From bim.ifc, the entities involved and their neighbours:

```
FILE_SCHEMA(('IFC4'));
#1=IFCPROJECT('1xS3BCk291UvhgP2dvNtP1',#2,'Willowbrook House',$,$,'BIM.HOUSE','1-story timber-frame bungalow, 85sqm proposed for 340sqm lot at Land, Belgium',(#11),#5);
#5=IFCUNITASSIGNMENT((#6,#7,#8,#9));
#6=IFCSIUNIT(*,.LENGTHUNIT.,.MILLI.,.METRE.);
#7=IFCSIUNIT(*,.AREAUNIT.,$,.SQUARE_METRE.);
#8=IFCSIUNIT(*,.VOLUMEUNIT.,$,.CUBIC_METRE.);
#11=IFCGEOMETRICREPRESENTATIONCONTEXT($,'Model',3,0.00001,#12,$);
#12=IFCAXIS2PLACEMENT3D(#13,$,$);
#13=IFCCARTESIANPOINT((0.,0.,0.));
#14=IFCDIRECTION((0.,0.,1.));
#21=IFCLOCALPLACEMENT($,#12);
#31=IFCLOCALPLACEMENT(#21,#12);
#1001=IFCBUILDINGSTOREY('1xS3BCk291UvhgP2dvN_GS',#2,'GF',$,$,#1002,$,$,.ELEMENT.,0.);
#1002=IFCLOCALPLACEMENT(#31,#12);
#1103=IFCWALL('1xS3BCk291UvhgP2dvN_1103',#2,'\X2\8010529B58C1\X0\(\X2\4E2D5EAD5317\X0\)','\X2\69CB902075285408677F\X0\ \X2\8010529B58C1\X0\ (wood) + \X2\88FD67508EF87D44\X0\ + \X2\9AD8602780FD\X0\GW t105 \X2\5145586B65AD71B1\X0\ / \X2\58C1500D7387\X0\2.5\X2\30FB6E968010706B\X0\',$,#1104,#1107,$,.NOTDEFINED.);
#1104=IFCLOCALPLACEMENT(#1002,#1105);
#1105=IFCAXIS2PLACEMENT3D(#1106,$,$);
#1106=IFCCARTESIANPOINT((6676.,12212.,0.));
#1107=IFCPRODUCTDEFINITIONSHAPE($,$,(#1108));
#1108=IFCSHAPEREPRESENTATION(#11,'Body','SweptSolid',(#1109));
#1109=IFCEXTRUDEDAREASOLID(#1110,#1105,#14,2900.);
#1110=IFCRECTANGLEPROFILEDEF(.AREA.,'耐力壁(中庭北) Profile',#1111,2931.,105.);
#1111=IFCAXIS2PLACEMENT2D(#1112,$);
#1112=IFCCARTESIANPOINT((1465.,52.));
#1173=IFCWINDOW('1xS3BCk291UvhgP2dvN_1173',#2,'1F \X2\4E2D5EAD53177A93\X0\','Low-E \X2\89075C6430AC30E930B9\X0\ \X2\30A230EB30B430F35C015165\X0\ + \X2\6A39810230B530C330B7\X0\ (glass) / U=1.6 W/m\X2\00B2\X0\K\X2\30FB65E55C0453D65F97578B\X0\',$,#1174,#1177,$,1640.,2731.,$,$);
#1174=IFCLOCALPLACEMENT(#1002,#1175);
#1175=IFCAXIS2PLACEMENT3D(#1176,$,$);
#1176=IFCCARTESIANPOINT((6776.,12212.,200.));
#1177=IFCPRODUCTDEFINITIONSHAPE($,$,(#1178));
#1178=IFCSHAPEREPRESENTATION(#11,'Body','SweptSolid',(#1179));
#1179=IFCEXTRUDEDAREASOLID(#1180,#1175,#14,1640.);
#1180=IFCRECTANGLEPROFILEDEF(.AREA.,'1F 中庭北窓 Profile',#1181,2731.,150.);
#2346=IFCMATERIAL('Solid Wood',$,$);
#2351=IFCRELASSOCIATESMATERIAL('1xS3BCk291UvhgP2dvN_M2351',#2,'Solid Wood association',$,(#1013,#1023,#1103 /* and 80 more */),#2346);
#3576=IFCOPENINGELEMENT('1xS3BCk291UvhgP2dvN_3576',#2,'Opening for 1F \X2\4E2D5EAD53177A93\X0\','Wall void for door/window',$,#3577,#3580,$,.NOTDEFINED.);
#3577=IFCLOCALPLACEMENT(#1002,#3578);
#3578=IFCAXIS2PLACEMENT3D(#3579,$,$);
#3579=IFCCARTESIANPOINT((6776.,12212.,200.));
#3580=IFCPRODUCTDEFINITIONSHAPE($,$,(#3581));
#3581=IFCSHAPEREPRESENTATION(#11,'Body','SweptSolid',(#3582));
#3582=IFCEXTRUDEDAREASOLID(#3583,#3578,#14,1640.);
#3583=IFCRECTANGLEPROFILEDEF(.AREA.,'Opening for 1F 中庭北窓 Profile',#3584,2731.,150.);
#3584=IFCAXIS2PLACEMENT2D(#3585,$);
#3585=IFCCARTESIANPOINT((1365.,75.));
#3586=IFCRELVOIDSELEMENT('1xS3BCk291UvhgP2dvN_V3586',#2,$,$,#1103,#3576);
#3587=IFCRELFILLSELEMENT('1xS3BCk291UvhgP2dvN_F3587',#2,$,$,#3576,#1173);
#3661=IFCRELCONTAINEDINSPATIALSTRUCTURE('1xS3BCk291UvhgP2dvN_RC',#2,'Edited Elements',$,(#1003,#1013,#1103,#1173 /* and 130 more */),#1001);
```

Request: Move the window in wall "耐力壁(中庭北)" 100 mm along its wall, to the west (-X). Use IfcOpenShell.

```python
import ifcopenshell
import ifcopenshell.api.geometry
import ifcopenshell.util.placement
import ifcopenshell.util.unit

model = ifcopenshell.open("bim.ifc")
unit_scale = ifcopenshell.util.unit.calculate_unit_scale(model)

window = model.by_guid("1xS3BCk291UvhgP2dvN_1173")
opening = window.FillsVoids[0].RelatingOpeningElement
wall = opening.VoidsElements[0].RelatingBuildingElement

wall_matrix = ifcopenshell.util.placement.get_local_placement(wall.ObjectPlacement)
shift = wall_matrix[:3, 0] * -0.1 / unit_scale
before = ifcopenshell.util.placement.get_local_placement(window.ObjectPlacement)[:3, 3].copy()

# The window is not placed relative to its opening, so move both.
for product in (opening, window):
    matrix = ifcopenshell.util.placement.get_local_placement(product.ObjectPlacement)
    matrix[:3, 3] += shift
    ifcopenshell.api.geometry.edit_object_placement(model, product=product, matrix=matrix, is_si=False)

after = ifcopenshell.util.placement.get_local_placement(window.ObjectPlacement)[:3, 3]
print("window moved by", (after - before).round(3) + 0.0)

model.write("bim_updated.ifc")
```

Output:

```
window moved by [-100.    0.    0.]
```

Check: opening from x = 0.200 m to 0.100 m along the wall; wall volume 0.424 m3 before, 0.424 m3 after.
